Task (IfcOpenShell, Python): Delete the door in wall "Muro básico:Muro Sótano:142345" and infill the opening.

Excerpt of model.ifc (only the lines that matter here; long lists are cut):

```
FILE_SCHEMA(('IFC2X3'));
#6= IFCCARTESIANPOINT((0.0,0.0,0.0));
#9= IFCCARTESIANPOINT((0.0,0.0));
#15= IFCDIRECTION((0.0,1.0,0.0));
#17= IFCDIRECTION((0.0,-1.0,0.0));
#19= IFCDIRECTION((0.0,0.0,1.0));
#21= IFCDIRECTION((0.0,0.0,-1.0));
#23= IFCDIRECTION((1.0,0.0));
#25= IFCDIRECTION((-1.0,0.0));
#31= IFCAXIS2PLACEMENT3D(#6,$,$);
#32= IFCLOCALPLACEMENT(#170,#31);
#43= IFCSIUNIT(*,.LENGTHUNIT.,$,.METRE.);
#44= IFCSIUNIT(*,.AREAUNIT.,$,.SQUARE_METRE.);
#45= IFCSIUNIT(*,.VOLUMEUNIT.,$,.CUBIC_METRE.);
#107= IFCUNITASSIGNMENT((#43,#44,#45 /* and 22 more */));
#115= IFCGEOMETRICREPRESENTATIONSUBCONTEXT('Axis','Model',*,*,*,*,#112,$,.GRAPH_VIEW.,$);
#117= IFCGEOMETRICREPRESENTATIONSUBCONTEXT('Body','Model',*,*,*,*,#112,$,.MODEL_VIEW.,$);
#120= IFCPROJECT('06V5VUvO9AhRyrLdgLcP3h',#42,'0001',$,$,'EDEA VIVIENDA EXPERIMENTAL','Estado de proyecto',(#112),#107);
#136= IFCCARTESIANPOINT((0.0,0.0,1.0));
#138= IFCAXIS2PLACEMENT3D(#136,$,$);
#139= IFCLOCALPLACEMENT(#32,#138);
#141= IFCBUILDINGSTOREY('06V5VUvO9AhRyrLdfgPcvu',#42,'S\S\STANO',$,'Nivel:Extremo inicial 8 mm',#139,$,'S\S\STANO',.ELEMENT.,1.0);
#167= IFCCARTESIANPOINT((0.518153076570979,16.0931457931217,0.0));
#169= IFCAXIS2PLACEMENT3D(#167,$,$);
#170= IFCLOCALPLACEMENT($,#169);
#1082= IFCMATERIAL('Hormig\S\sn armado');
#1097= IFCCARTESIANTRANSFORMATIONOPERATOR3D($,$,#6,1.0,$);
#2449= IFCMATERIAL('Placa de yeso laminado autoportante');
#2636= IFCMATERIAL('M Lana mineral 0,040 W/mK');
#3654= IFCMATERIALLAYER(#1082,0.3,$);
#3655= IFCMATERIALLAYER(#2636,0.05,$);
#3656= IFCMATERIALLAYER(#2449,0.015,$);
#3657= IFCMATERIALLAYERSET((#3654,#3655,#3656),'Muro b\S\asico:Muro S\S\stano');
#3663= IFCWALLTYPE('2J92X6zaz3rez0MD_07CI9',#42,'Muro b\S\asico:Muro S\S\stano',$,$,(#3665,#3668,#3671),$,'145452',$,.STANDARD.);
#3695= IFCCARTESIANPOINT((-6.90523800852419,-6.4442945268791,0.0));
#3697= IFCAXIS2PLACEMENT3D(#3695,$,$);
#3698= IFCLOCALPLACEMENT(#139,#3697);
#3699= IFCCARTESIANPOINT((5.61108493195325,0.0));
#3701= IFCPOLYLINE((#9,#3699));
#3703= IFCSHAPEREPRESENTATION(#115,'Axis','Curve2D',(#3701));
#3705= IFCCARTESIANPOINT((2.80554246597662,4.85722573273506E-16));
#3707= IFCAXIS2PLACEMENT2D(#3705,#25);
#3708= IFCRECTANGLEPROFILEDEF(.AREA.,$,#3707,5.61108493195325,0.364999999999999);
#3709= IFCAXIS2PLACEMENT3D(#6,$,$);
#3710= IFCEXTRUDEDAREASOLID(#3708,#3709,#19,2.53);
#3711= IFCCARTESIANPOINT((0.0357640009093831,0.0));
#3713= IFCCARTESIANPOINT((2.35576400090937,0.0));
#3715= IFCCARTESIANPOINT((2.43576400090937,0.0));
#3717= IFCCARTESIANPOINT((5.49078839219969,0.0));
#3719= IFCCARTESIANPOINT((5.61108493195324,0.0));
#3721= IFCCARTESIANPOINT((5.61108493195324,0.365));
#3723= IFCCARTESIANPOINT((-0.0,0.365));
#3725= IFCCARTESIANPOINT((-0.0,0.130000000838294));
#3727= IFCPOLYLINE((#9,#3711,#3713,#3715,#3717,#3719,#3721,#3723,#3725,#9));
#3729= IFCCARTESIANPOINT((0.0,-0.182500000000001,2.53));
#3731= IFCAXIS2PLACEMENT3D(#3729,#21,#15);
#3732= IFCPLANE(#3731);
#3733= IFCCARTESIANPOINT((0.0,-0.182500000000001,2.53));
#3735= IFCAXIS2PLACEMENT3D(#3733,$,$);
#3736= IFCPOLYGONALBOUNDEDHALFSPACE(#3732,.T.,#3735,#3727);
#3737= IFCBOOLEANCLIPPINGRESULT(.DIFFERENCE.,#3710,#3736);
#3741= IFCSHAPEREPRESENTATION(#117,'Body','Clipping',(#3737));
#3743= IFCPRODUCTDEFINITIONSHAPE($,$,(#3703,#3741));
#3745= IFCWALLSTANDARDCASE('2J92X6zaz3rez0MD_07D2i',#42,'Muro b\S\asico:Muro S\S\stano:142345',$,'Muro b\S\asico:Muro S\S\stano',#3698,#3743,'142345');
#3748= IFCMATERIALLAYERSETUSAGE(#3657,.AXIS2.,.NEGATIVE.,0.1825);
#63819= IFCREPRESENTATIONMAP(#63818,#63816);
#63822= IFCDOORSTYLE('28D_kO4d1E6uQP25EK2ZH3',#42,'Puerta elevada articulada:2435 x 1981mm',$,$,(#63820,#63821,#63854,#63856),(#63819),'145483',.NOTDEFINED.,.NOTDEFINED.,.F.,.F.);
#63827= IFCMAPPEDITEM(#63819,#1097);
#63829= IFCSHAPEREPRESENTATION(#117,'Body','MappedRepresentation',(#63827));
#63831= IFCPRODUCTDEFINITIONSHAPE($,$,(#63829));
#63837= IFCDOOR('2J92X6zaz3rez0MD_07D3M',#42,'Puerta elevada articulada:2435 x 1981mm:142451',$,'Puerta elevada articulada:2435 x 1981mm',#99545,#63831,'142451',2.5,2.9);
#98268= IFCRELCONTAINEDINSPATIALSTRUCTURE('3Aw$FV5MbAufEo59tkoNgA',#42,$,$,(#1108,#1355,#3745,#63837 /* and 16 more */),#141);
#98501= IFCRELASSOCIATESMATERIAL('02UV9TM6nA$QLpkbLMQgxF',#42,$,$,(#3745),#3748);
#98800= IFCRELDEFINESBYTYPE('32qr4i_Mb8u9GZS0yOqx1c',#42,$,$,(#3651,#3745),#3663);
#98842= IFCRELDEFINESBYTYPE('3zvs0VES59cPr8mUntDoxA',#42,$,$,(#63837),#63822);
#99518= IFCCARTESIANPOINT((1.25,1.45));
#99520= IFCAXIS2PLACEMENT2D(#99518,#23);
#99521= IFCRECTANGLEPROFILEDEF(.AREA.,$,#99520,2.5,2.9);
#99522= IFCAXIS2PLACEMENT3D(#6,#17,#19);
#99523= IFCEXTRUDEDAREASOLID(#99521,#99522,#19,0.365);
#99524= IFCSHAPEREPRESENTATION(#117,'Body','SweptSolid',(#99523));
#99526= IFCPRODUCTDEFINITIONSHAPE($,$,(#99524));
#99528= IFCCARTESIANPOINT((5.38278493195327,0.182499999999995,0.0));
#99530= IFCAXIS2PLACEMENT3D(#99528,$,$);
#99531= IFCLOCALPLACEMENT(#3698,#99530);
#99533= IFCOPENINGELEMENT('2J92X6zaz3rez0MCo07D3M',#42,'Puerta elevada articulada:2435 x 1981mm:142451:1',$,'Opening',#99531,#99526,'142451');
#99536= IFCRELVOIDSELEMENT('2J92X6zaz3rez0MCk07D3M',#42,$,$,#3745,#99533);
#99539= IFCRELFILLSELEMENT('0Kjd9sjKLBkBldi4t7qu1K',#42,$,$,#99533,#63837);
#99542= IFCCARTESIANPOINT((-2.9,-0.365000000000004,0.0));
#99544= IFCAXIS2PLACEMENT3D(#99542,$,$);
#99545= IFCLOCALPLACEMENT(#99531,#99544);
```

```python
import ifcopenshell
import ifcopenshell.api.feature
import ifcopenshell.api.root
import ifcopenshell.geom
import ifcopenshell.util.shape

model = ifcopenshell.open("model.ifc")
settings = ifcopenshell.geom.settings()


def volume(element):
    """Net volume in cubic metres, openings subtracted."""
    shape = ifcopenshell.geom.create_shape(settings, element)
    return ifcopenshell.util.shape.get_volume(shape.geometry)


door = model.by_id(63837)
opening = door.FillsVoids[0].RelatingOpeningElement
wall = opening.VoidsElements[0].RelatingBuildingElement
before = volume(wall)

ifcopenshell.api.root.remove_product(model, product=door)
ifcopenshell.api.feature.remove_feature(model, feature=opening)

after = volume(wall)

print(f"wall volume {before:.3f} -> {after:.3f} m3")

model.write("model-out.ifc")
```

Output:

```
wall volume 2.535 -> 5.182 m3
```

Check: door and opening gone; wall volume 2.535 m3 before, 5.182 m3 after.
